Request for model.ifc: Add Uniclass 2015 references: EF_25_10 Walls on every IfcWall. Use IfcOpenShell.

First a look at what the model holds.

```python
import ifcopenshell

model = ifcopenshell.open("model.ifc")
print(model.schema)
print("classifications:", [c.Name for c in model.by_type("IfcClassification")])
for ifc_class in ("IfcDoor", "IfcRoof", "IfcStair", "IfcWall", "IfcWindow"):
    print(ifc_class, len(model.by_type(ifc_class)))
```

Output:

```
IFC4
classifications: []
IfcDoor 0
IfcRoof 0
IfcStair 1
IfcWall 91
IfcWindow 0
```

```python
import ifcopenshell
import ifcopenshell.api.classification

model = ifcopenshell.open("model.ifc")

system = ifcopenshell.api.classification.add_classification(model, classification="Uniclass 2015")

codes = {
    "IfcWall": ("EF_25_10", "Walls"),
}
for ifc_class, (code, name) in codes.items():
    products = model.by_type(ifc_class)
    ifcopenshell.api.classification.add_reference(
        model, products=products, classification=system, identification=code, name=name
    )
    print(code, len(products))

model.write("model-out.ifc")
```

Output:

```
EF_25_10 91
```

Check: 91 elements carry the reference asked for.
